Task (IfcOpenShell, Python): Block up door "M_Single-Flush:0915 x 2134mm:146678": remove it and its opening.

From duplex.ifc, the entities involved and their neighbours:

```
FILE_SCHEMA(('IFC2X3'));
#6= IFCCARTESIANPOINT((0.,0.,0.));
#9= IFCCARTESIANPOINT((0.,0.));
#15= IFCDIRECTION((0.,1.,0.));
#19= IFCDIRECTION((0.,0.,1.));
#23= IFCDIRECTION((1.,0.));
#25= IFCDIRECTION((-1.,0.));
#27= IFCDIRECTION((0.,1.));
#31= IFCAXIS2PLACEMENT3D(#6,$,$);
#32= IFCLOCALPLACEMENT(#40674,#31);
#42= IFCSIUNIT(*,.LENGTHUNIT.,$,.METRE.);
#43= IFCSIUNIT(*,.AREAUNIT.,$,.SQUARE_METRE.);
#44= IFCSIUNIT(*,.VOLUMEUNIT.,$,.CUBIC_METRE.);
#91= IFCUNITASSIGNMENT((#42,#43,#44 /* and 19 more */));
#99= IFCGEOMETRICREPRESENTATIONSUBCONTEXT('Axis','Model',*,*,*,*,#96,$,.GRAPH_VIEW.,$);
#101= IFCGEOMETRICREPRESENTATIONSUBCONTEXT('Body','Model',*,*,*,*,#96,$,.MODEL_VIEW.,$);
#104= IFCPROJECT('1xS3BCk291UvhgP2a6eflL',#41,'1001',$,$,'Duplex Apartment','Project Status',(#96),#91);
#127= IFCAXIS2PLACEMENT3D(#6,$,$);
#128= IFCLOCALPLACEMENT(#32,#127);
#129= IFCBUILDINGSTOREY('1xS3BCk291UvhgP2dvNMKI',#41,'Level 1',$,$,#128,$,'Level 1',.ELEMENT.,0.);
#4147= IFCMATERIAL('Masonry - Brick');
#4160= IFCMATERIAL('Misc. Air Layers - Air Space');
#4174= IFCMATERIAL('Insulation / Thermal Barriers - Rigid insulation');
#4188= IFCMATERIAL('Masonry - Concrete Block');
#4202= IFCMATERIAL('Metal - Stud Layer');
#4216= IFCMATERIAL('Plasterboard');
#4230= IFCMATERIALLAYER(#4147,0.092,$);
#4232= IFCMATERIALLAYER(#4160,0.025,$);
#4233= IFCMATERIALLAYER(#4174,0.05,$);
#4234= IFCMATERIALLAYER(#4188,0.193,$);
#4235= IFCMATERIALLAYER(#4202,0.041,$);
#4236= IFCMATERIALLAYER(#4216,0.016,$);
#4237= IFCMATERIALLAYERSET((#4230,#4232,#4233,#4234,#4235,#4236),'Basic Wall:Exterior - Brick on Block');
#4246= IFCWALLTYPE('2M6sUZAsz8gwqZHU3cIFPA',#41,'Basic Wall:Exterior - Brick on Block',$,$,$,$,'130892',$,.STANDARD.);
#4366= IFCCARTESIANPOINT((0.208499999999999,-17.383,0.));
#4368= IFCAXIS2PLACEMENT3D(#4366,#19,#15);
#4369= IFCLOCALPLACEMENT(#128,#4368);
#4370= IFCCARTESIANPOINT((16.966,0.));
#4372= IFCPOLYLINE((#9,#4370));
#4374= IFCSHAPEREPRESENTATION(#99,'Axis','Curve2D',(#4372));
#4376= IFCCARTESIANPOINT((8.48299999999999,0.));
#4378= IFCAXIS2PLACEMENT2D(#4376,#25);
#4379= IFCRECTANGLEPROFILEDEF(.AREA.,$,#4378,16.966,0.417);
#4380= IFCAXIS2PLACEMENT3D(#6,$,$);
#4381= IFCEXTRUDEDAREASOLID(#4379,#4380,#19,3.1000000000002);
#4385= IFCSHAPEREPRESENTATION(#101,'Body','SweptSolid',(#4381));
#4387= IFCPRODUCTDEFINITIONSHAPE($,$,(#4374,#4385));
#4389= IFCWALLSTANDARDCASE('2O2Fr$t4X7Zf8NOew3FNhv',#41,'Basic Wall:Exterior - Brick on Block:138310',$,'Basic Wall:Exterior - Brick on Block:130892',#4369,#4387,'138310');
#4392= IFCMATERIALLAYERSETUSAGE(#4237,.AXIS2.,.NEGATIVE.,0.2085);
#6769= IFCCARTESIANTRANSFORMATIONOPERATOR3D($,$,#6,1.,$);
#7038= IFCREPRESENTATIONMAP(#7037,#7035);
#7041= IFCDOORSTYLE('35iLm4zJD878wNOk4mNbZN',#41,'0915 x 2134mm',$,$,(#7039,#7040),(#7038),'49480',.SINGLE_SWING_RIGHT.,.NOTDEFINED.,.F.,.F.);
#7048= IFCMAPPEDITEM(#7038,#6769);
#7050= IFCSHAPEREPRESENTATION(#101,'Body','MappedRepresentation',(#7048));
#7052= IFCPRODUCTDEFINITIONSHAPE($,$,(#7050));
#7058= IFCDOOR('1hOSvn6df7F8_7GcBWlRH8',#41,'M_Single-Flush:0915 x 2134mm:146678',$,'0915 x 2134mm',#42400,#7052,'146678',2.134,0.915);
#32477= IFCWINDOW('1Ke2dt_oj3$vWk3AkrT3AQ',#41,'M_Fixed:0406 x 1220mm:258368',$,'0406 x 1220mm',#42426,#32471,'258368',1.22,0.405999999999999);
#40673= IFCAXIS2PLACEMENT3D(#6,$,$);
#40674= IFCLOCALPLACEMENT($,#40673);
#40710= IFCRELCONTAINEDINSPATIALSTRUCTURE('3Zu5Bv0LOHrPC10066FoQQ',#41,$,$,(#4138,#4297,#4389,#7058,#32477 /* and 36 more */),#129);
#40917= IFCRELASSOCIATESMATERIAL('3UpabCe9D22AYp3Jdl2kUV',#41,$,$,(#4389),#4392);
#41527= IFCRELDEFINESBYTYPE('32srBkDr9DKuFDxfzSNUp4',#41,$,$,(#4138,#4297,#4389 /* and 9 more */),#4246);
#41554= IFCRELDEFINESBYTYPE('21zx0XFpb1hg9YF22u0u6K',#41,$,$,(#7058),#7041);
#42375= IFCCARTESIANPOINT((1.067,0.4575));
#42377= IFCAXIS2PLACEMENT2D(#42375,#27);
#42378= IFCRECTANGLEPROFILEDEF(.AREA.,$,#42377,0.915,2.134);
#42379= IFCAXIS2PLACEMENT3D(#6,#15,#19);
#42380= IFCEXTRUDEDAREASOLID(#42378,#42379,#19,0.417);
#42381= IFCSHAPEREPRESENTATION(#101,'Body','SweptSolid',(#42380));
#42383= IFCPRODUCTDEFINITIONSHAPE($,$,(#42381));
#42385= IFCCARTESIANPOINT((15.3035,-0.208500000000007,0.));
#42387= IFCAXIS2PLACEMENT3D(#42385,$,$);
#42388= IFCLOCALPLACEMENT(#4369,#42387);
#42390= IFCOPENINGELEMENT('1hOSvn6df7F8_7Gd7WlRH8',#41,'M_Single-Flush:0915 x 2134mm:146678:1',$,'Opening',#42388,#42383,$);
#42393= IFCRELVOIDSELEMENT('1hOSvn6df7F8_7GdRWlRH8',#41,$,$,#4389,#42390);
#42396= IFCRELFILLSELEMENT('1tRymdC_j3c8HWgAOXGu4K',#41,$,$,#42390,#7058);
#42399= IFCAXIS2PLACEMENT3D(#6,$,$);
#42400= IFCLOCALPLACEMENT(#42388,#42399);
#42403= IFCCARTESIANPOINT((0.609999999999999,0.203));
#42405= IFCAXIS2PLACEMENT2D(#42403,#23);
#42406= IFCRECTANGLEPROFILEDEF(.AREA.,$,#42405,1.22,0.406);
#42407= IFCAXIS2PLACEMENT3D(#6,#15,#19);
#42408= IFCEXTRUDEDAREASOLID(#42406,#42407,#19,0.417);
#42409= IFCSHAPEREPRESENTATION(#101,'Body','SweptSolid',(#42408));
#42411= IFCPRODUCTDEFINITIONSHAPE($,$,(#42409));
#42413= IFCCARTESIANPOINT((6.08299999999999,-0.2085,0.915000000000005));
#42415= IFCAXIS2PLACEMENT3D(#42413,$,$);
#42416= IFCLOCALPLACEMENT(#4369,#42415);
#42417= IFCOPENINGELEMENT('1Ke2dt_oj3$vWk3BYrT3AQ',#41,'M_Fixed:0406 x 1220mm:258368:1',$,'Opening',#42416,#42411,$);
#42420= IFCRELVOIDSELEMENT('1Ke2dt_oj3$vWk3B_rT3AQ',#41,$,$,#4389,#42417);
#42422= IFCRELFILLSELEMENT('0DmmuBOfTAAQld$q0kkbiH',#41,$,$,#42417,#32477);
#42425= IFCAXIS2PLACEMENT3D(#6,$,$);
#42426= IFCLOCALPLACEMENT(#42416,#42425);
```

```python
import ifcopenshell
import ifcopenshell.api.feature
import ifcopenshell.api.root
import ifcopenshell.geom
import ifcopenshell.util.shape

model = ifcopenshell.open("duplex.ifc")
settings = ifcopenshell.geom.settings()


def volume(element):
    """Net volume in cubic metres, openings subtracted."""
    shape = ifcopenshell.geom.create_shape(settings, element)
    return ifcopenshell.util.shape.get_volume(shape.geometry)


door = model.by_guid("1hOSvn6df7F8_7GcBWlRH8")
opening = door.FillsVoids[0].RelatingOpeningElement
wall = opening.VoidsElements[0].RelatingBuildingElement
before = volume(wall)

ifcopenshell.api.root.remove_product(model, product=door)
ifcopenshell.api.feature.remove_feature(model, feature=opening)

after = volume(wall)

print(f"wall volume {before:.3f} -> {after:.3f} m3")

model.write("duplex_v2.ifc")
```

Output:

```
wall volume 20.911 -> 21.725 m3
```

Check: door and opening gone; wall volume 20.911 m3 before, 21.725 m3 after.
